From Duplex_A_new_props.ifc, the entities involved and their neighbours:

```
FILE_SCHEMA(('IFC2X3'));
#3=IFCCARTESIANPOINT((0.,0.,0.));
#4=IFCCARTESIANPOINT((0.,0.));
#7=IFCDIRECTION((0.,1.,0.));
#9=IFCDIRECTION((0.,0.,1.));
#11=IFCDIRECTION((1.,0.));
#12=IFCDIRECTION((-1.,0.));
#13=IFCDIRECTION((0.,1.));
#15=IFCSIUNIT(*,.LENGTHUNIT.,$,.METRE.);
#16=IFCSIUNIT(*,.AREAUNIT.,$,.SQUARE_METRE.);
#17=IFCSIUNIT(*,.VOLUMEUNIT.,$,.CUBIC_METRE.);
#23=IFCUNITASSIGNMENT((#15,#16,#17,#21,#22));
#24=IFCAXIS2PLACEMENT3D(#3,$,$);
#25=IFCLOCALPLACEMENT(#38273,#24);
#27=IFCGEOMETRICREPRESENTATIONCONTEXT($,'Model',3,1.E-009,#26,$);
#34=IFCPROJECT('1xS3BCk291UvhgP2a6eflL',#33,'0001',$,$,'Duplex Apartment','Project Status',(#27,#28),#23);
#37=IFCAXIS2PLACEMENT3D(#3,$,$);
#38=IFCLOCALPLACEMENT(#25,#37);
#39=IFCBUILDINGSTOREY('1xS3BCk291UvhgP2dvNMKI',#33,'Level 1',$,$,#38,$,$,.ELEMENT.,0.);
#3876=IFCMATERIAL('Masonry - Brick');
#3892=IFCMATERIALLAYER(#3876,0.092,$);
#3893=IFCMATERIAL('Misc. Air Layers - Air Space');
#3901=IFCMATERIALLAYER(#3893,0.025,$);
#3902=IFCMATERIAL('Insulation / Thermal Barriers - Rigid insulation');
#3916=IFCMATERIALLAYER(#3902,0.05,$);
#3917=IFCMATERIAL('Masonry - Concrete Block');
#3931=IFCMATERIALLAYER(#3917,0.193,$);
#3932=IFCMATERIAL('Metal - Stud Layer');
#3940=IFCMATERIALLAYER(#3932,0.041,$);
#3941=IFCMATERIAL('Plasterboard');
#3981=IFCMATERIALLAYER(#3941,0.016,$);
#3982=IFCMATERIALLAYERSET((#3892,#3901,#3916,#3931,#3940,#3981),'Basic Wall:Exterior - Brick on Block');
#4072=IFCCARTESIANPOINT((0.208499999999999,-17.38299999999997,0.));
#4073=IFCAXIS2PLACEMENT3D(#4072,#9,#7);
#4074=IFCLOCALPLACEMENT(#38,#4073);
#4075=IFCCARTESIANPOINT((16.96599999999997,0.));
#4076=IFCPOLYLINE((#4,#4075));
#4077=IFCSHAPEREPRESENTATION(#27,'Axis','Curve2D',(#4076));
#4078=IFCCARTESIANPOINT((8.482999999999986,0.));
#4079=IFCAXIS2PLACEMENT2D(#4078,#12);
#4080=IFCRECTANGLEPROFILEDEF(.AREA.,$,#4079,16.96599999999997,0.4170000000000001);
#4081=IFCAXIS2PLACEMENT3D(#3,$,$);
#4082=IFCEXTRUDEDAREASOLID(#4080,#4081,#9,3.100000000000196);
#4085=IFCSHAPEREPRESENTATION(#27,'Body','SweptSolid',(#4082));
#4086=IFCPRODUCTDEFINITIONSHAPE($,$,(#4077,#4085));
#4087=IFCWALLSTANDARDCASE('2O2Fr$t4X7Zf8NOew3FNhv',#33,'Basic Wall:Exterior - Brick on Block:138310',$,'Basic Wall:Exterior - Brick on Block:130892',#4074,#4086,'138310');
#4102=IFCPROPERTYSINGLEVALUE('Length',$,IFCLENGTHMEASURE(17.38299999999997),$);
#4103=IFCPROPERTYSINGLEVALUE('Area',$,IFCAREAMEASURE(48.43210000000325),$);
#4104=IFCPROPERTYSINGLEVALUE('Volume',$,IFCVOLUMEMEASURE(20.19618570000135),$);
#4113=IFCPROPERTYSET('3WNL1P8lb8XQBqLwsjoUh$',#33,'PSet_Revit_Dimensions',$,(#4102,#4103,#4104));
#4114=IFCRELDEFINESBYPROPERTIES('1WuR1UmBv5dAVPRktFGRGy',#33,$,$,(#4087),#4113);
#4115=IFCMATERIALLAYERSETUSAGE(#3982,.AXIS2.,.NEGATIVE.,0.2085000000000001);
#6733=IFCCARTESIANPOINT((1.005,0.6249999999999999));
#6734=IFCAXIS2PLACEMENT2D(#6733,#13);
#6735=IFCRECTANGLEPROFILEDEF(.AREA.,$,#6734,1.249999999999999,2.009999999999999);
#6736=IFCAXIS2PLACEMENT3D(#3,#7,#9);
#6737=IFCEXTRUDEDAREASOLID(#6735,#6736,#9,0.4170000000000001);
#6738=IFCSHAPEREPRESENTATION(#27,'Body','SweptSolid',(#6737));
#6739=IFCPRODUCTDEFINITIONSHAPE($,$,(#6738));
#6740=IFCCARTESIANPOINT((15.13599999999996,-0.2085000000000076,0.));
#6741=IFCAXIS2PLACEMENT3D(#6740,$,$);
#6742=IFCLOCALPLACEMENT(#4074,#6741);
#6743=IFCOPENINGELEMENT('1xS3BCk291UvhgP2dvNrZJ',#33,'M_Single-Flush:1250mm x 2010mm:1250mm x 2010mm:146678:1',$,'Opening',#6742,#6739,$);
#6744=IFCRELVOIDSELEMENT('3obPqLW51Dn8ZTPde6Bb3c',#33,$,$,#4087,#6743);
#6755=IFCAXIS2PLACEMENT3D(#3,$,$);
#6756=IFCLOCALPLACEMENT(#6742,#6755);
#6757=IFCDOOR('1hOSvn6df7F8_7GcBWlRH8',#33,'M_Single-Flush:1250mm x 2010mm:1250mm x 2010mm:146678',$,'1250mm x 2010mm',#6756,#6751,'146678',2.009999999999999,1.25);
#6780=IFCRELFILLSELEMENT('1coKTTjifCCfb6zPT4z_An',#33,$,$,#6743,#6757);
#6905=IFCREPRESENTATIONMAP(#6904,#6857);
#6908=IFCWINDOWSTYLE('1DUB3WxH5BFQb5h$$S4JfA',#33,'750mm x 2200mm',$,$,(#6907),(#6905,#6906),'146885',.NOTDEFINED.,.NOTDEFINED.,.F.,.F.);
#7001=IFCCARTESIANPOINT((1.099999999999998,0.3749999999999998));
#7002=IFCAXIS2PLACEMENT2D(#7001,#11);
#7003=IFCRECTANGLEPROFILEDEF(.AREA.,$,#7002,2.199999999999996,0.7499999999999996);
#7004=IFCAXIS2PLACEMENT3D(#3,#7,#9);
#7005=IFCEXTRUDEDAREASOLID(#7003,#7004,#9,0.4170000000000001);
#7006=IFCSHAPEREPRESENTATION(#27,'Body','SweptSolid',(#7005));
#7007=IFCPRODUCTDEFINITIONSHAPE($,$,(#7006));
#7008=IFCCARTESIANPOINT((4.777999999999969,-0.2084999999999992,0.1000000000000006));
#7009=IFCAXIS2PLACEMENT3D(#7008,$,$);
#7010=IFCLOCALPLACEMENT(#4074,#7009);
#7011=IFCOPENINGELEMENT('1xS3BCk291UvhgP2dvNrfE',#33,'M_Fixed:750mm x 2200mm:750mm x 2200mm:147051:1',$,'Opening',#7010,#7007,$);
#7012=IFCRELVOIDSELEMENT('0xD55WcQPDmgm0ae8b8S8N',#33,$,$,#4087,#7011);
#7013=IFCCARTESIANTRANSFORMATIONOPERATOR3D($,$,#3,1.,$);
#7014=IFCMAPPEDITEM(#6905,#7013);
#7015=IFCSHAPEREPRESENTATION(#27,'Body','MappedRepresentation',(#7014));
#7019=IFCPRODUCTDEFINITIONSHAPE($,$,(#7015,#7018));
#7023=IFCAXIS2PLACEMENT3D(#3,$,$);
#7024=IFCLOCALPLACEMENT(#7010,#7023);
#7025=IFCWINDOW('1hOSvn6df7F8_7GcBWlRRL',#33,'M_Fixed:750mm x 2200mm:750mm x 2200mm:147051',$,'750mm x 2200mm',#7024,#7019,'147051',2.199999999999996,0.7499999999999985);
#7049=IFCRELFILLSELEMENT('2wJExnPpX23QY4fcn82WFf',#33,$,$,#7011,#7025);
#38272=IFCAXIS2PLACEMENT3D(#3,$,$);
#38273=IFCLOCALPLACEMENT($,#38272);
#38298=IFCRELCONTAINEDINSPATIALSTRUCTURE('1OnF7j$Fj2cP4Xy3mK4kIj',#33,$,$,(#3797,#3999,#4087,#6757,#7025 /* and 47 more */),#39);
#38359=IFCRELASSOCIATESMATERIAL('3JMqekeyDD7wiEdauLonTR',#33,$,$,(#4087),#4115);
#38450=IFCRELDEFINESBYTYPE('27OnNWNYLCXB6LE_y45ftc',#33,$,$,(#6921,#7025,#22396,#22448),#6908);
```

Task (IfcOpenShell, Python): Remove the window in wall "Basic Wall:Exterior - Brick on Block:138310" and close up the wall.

```python
import ifcopenshell
import ifcopenshell.api.feature
import ifcopenshell.api.pset
import ifcopenshell.api.root
import ifcopenshell.geom
import ifcopenshell.util.element
import ifcopenshell.util.shape
import ifcopenshell.util.unit

model = ifcopenshell.open("Duplex_A_new_props.ifc")
area_scale = ifcopenshell.util.unit.calculate_unit_scale(model, "AREAUNIT")
volume_scale = ifcopenshell.util.unit.calculate_unit_scale(model, "VOLUMEUNIT")
settings = ifcopenshell.geom.settings()


def volume(element):
    """Net volume in cubic metres, openings subtracted."""
    shape = ifcopenshell.geom.create_shape(settings, element)
    return ifcopenshell.util.shape.get_volume(shape.geometry)


window = model.by_guid("1hOSvn6df7F8_7GcBWlRRL")
opening = window.FillsVoids[0].RelatingOpeningElement
wall = opening.VoidsElements[0].RelatingBuildingElement
before = volume(wall)

ifcopenshell.api.root.remove_product(model, product=window)
ifcopenshell.api.feature.remove_feature(model, feature=opening)

after = volume(wall)
thickness = 0.417  # wall thickness in metres

# Update the wall's stored quantities.
pset = model.by_id(ifcopenshell.util.element.get_pset(wall, "PSet_Revit_Dimensions", should_inherit=False)["id"])
ifcopenshell.api.pset.edit_pset(model, pset=pset, properties={
    "Area": model.create_entity("IfcAreaMeasure", after / thickness / area_scale),
    "Volume": model.create_entity("IfcVolumeMeasure", after / volume_scale),
})

print(f"wall volume {before:.3f} -> {after:.3f} m3")

model.write("Duplex_A_new_props_updated.ifc")
```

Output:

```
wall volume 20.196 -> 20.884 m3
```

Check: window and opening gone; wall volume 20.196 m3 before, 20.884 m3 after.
